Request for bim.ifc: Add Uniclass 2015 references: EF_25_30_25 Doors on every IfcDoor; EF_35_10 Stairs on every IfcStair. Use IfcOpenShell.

First a look at what the model holds.

```python
import ifcopenshell

model = ifcopenshell.open("bim.ifc")
print(model.schema)
print("classifications:", [c.Name for c in model.by_type("IfcClassification")])
for ifc_class in ("IfcDoor", "IfcRoof", "IfcStair", "IfcWall", "IfcWindow"):
    print(ifc_class, len(model.by_type(ifc_class)))
```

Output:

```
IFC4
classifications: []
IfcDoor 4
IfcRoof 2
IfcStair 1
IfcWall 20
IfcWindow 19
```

```python
import ifcopenshell
import ifcopenshell.api.classification

model = ifcopenshell.open("bim.ifc")

system = ifcopenshell.api.classification.add_classification(model, classification="Uniclass 2015")

codes = {
    "IfcDoor": ("EF_25_30_25", "Doors"),
    "IfcStair": ("EF_35_10", "Stairs"),
}
for ifc_class, (code, name) in codes.items():
    products = model.by_type(ifc_class)
    ifcopenshell.api.classification.add_reference(
        model, products=products, classification=system, identification=code, name=name
    )
    print(code, len(products))

model.write("bim_updated.ifc")
```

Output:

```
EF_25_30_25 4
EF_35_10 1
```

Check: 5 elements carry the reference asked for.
